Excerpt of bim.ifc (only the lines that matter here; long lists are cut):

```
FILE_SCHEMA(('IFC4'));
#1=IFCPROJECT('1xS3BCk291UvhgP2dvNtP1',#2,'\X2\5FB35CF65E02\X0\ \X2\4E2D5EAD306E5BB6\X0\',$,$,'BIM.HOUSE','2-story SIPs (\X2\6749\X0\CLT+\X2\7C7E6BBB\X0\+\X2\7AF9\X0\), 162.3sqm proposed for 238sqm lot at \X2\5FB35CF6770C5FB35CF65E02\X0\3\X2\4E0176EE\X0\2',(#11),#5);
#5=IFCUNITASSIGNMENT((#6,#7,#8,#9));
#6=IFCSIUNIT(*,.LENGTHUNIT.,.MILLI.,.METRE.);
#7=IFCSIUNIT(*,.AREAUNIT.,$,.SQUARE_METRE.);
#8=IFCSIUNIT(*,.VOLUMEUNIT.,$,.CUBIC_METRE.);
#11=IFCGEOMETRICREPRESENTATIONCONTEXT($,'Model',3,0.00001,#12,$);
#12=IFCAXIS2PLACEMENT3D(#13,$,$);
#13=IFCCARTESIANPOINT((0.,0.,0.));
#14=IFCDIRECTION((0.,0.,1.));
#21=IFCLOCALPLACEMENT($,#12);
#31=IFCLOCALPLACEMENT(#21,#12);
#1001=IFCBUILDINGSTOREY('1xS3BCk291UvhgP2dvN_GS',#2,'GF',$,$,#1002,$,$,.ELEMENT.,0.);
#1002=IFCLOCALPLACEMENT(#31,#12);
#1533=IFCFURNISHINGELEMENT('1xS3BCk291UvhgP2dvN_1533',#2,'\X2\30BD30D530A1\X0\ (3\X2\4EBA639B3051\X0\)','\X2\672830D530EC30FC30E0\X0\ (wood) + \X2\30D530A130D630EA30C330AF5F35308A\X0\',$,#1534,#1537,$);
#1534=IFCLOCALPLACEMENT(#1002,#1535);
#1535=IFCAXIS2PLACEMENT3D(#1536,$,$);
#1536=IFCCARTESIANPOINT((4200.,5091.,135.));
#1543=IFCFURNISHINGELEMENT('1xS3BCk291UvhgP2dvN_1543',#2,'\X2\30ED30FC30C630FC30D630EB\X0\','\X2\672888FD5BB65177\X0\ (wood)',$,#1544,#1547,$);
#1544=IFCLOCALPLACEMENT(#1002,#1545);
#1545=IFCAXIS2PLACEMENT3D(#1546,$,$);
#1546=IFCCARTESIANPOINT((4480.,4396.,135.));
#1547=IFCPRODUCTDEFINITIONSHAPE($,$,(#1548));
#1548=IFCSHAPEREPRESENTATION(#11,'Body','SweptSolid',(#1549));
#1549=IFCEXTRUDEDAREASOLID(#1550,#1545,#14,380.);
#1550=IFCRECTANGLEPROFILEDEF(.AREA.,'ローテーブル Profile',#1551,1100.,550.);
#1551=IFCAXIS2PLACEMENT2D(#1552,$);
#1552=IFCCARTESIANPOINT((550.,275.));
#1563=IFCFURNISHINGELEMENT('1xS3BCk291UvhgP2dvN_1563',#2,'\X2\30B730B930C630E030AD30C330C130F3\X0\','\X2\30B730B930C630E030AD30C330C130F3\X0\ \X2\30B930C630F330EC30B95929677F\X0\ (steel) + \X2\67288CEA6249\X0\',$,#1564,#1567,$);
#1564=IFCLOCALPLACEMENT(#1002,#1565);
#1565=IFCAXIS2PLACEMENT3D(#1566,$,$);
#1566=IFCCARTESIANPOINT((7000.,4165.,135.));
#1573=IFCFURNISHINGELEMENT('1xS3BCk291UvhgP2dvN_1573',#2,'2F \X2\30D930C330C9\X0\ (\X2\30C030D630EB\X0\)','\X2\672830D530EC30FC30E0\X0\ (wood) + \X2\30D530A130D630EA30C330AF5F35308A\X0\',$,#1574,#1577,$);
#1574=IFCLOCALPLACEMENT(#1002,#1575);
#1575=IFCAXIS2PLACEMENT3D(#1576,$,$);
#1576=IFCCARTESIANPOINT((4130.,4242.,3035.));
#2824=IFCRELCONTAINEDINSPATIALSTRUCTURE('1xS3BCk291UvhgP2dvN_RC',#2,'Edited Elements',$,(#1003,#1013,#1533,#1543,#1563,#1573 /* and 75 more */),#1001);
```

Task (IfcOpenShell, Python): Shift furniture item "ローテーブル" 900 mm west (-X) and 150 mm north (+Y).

```python
import ifcopenshell
import ifcopenshell.api.geometry
import ifcopenshell.util.placement
import ifcopenshell.util.unit

model = ifcopenshell.open("bim.ifc")
unit_scale = ifcopenshell.util.unit.calculate_unit_scale(model)

item = model.by_id(1543)
matrix = ifcopenshell.util.placement.get_local_placement(item.ObjectPlacement)
matrix[0, 3] -= 0.9 / unit_scale
matrix[1, 3] += 0.15 / unit_scale
ifcopenshell.api.geometry.edit_object_placement(model, product=item, matrix=matrix, is_si=False)

print(ifcopenshell.util.placement.get_local_placement(item.ObjectPlacement).round(3) + 0.0)

model.write("bim_rev.ifc")
```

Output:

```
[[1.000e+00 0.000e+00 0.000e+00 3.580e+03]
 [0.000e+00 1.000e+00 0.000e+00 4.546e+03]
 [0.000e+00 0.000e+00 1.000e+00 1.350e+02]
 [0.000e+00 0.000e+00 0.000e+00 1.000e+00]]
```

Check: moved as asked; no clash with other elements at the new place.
